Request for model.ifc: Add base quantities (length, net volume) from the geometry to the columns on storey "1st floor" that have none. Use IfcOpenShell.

First a look at what the model holds.

```python
import ifcopenshell
import ifcopenshell.util.element
import ifcopenshell.util.unit

model = ifcopenshell.open("model.ifc")
print(model.schema)
for unit_type in ("LENGTHUNIT", "AREAUNIT", "VOLUMEUNIT"):
    print(unit_type, ifcopenshell.util.unit.calculate_unit_scale(model, unit_type))
storey = next(s for s in model.by_type("IfcBuildingStorey") if s.Name == "1st floor")
columns = [e for e in ifcopenshell.util.element.get_decomposition(storey) if e.is_a("IfcColumn")]
for e in sorted(columns, key=lambda e: e.id()):
    print(e.id(), e.is_a(), e.Name, list(ifcopenshell.util.element.get_psets(e, qtos_only=True)), sep=" | ")
```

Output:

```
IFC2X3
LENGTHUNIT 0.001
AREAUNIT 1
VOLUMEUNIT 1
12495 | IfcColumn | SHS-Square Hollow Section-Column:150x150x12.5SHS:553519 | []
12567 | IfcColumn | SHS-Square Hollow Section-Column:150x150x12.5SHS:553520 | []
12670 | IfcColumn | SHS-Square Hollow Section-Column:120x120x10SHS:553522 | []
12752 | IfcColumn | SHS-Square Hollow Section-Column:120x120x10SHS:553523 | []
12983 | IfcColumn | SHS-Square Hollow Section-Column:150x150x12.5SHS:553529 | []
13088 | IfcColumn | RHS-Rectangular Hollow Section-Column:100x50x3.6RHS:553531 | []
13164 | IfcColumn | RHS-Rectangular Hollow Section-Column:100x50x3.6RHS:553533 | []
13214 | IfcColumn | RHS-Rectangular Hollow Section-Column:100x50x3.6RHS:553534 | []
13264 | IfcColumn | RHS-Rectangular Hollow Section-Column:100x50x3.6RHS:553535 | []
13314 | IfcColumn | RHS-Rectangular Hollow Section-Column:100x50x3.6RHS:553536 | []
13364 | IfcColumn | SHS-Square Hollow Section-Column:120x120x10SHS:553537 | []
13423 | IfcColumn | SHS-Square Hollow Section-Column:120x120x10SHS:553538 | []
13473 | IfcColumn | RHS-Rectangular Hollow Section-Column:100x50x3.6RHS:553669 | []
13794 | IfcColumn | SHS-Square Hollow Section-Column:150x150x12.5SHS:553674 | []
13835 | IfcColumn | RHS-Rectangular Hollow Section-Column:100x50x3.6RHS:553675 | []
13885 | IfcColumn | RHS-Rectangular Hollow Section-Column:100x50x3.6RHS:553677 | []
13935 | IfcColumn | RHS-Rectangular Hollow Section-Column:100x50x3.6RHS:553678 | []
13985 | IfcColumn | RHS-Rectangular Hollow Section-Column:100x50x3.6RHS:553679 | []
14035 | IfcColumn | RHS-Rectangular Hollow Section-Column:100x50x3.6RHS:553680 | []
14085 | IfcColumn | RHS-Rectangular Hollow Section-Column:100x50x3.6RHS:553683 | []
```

```python
import ifcopenshell
import ifcopenshell.api.pset
import ifcopenshell.geom
import ifcopenshell.util.element
import ifcopenshell.util.shape
import ifcopenshell.util.unit

model = ifcopenshell.open("model.ifc")
unit_scale = ifcopenshell.util.unit.calculate_unit_scale(model)
volume_scale = ifcopenshell.util.unit.calculate_unit_scale(model, "VOLUMEUNIT")
settings = ifcopenshell.geom.settings()

storey = next(s for s in model.by_type("IfcBuildingStorey") if s.Name == "1st floor")
columns = [e for e in ifcopenshell.util.element.get_decomposition(storey) if e.is_a("IfcColumn")]

for e in sorted(columns, key=lambda e: e.id()):
    if ifcopenshell.util.element.get_psets(e, qtos_only=True, should_inherit=False):
        continue
    # Geometry comes back in metres, in the element's own axes.
    shape = ifcopenshell.geom.create_shape(settings, e)
    values = {
        "Length": ifcopenshell.util.shape.get_z(shape.geometry) / unit_scale,
        "NetVolume": ifcopenshell.util.shape.get_volume(shape.geometry) / volume_scale,
    }
    qto = ifcopenshell.api.pset.add_qto(model, product=e, name="BaseQuantities")
    ifcopenshell.api.pset.edit_qto(model, qto=qto, properties=values)
    print(e.id(), {k: round(v, 3) for k, v in values.items()})

model.write("model_v2.ifc")
```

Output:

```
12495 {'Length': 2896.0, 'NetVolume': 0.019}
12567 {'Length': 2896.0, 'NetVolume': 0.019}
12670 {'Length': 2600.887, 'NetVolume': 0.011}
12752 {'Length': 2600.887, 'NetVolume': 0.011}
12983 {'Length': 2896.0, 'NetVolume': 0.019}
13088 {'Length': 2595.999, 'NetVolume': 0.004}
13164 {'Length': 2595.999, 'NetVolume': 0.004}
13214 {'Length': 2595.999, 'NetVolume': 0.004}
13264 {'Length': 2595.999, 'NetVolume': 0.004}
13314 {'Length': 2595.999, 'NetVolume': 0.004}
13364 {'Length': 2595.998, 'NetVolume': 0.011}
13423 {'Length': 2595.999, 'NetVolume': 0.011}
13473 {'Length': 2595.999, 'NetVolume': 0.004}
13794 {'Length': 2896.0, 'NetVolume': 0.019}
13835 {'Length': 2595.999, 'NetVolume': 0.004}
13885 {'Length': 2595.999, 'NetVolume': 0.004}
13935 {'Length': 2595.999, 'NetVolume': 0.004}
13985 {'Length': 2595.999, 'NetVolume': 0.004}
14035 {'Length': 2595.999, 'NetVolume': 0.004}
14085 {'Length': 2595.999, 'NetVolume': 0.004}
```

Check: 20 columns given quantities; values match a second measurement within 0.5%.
